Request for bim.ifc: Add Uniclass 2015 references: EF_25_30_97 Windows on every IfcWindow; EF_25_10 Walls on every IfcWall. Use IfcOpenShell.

First a look at what the model holds.

```python
import ifcopenshell

model = ifcopenshell.open("bim.ifc")
print(model.schema)
print("classifications:", [c.Name for c in model.by_type("IfcClassification")])
for ifc_class in ("IfcDoor", "IfcRoof", "IfcStair", "IfcWall", "IfcWindow"):
    print(ifc_class, len(model.by_type(ifc_class)))
```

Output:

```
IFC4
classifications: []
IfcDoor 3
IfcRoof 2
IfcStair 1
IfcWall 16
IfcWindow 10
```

```python
import ifcopenshell
import ifcopenshell.api.classification

model = ifcopenshell.open("bim.ifc")

system = ifcopenshell.api.classification.add_classification(model, classification="Uniclass 2015")

codes = {
    "IfcWindow": ("EF_25_30_97", "Windows"),
    "IfcWall": ("EF_25_10", "Walls"),
}
for ifc_class, (code, name) in codes.items():
    products = model.by_type(ifc_class)
    ifcopenshell.api.classification.add_reference(
        model, products=products, classification=system, identification=code, name=name
    )
    print(code, len(products))

model.write("bim_v2.ifc")
```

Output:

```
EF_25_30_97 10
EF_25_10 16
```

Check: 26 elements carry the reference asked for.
